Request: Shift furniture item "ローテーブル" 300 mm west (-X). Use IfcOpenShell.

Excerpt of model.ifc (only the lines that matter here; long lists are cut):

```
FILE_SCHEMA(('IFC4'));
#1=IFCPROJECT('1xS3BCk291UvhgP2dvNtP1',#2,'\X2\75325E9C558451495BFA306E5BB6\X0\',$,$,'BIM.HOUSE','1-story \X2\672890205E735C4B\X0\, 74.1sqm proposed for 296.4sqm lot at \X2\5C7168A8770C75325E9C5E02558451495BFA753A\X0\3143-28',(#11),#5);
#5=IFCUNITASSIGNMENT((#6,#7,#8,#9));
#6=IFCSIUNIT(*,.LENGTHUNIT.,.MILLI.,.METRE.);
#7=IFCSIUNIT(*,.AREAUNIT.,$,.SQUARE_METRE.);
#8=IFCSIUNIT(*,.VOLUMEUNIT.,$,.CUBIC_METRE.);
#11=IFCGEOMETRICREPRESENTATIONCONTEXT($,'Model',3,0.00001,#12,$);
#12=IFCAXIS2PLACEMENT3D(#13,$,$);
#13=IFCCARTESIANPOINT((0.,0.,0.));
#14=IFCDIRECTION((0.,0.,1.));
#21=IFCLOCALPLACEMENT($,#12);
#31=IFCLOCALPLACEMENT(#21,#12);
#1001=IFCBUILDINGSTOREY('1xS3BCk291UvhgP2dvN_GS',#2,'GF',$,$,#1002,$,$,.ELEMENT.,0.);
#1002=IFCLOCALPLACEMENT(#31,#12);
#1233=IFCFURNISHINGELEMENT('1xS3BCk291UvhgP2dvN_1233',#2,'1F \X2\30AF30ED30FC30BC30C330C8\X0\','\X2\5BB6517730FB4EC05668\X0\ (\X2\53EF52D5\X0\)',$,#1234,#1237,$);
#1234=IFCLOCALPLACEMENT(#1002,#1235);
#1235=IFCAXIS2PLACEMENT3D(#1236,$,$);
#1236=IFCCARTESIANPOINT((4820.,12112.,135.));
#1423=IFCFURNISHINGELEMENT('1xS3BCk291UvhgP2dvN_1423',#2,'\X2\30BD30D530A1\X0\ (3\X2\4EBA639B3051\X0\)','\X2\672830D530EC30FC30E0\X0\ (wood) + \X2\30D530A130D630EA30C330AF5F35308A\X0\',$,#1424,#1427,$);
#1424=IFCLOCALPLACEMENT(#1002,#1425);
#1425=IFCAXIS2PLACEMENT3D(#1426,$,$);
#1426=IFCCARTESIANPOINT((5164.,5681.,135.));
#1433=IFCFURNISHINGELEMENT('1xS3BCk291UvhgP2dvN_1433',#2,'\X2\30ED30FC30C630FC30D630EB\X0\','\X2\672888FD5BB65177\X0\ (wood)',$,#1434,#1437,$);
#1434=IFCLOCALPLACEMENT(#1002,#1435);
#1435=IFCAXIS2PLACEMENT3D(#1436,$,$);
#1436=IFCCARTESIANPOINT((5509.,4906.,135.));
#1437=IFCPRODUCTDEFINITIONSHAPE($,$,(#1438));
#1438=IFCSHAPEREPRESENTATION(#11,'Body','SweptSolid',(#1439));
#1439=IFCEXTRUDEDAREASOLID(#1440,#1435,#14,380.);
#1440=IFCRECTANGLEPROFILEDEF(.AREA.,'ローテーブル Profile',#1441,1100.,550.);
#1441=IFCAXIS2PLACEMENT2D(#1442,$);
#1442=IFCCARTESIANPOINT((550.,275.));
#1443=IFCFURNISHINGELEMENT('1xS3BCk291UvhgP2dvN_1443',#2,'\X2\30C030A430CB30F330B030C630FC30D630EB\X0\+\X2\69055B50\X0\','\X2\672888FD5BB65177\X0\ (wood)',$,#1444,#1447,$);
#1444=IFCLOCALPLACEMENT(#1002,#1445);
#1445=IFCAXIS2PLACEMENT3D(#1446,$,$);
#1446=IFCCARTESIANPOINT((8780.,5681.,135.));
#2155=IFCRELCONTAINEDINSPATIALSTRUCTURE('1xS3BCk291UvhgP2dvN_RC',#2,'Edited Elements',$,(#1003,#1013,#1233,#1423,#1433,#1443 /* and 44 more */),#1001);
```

```python
import ifcopenshell
import ifcopenshell.api.geometry
import ifcopenshell.util.placement
import ifcopenshell.util.unit

model = ifcopenshell.open("model.ifc")
unit_scale = ifcopenshell.util.unit.calculate_unit_scale(model)

item = model.by_guid("1xS3BCk291UvhgP2dvN_1433")
matrix = ifcopenshell.util.placement.get_local_placement(item.ObjectPlacement)
matrix[0, 3] -= 0.3 / unit_scale
ifcopenshell.api.geometry.edit_object_placement(model, product=item, matrix=matrix, is_si=False)

print(ifcopenshell.util.placement.get_local_placement(item.ObjectPlacement).round(3) + 0.0)

model.write("model_updated.ifc")
```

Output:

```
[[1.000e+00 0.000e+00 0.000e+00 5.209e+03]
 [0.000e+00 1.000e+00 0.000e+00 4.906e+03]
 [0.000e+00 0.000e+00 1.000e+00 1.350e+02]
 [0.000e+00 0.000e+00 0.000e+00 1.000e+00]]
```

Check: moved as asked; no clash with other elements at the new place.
